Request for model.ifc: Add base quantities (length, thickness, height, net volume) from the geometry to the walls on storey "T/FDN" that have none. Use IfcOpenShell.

First a look at what the model holds.

```python
import ifcopenshell
import ifcopenshell.util.element
import ifcopenshell.util.unit

model = ifcopenshell.open("model.ifc")
print(model.schema)
for unit_type in ("LENGTHUNIT", "AREAUNIT", "VOLUMEUNIT"):
    print(unit_type, ifcopenshell.util.unit.calculate_unit_scale(model, unit_type))
storey = next(s for s in model.by_type("IfcBuildingStorey") if s.Name == "T/FDN")
walls = [e for e in ifcopenshell.util.element.get_decomposition(storey) if e.is_a("IfcWall")]
for e in sorted(walls, key=lambda e: e.id()):
    print(e.id(), e.is_a(), e.Name, list(ifcopenshell.util.element.get_psets(e, qtos_only=True)), sep=" | ")
```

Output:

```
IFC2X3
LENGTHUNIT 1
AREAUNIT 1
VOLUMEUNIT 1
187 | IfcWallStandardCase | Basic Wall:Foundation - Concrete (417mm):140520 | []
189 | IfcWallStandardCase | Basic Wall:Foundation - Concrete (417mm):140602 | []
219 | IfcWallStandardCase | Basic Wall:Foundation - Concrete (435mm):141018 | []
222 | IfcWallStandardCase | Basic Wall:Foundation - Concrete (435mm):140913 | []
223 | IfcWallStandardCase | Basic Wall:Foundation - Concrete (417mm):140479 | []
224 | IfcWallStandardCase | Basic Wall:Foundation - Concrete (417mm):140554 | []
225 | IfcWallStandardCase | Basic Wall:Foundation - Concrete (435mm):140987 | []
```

```python
import ifcopenshell
import ifcopenshell.api.pset
import ifcopenshell.geom
import ifcopenshell.util.element
import ifcopenshell.util.shape
import ifcopenshell.util.unit

model = ifcopenshell.open("model.ifc")
unit_scale = ifcopenshell.util.unit.calculate_unit_scale(model)
volume_scale = ifcopenshell.util.unit.calculate_unit_scale(model, "VOLUMEUNIT")
settings = ifcopenshell.geom.settings()

storey = next(s for s in model.by_type("IfcBuildingStorey") if s.Name == "T/FDN")
walls = [e for e in ifcopenshell.util.element.get_decomposition(storey) if e.is_a("IfcWall")]

for e in sorted(walls, key=lambda e: e.id()):
    if ifcopenshell.util.element.get_psets(e, qtos_only=True, should_inherit=False):
        continue
    # Geometry comes back in metres, in the element's own axes.
    shape = ifcopenshell.geom.create_shape(settings, e)
    values = {
        "Length": ifcopenshell.util.shape.get_x(shape.geometry) / unit_scale,
        "Width": ifcopenshell.util.shape.get_y(shape.geometry) / unit_scale,
        "Height": ifcopenshell.util.shape.get_z(shape.geometry) / unit_scale,
        "NetVolume": ifcopenshell.util.shape.get_volume(shape.geometry) / volume_scale,
    }
    qto = ifcopenshell.api.pset.add_qto(model, product=e, name="BaseQuantities")
    ifcopenshell.api.pset.edit_qto(model, qto=qto, properties=values)
    print(e.id(), {k: round(v, 3) for k, v in values.items()})

model.write("model_v2.ifc")
```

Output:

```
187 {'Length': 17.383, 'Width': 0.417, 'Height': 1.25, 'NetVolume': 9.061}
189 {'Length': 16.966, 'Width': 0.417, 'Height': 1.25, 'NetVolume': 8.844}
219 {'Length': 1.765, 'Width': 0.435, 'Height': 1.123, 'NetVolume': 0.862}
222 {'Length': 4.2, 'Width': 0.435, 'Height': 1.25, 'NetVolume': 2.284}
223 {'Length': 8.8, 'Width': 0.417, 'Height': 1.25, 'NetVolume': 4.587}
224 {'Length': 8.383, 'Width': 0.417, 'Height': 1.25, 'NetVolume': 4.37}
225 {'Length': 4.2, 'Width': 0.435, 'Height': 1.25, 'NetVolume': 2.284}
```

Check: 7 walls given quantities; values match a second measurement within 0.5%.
